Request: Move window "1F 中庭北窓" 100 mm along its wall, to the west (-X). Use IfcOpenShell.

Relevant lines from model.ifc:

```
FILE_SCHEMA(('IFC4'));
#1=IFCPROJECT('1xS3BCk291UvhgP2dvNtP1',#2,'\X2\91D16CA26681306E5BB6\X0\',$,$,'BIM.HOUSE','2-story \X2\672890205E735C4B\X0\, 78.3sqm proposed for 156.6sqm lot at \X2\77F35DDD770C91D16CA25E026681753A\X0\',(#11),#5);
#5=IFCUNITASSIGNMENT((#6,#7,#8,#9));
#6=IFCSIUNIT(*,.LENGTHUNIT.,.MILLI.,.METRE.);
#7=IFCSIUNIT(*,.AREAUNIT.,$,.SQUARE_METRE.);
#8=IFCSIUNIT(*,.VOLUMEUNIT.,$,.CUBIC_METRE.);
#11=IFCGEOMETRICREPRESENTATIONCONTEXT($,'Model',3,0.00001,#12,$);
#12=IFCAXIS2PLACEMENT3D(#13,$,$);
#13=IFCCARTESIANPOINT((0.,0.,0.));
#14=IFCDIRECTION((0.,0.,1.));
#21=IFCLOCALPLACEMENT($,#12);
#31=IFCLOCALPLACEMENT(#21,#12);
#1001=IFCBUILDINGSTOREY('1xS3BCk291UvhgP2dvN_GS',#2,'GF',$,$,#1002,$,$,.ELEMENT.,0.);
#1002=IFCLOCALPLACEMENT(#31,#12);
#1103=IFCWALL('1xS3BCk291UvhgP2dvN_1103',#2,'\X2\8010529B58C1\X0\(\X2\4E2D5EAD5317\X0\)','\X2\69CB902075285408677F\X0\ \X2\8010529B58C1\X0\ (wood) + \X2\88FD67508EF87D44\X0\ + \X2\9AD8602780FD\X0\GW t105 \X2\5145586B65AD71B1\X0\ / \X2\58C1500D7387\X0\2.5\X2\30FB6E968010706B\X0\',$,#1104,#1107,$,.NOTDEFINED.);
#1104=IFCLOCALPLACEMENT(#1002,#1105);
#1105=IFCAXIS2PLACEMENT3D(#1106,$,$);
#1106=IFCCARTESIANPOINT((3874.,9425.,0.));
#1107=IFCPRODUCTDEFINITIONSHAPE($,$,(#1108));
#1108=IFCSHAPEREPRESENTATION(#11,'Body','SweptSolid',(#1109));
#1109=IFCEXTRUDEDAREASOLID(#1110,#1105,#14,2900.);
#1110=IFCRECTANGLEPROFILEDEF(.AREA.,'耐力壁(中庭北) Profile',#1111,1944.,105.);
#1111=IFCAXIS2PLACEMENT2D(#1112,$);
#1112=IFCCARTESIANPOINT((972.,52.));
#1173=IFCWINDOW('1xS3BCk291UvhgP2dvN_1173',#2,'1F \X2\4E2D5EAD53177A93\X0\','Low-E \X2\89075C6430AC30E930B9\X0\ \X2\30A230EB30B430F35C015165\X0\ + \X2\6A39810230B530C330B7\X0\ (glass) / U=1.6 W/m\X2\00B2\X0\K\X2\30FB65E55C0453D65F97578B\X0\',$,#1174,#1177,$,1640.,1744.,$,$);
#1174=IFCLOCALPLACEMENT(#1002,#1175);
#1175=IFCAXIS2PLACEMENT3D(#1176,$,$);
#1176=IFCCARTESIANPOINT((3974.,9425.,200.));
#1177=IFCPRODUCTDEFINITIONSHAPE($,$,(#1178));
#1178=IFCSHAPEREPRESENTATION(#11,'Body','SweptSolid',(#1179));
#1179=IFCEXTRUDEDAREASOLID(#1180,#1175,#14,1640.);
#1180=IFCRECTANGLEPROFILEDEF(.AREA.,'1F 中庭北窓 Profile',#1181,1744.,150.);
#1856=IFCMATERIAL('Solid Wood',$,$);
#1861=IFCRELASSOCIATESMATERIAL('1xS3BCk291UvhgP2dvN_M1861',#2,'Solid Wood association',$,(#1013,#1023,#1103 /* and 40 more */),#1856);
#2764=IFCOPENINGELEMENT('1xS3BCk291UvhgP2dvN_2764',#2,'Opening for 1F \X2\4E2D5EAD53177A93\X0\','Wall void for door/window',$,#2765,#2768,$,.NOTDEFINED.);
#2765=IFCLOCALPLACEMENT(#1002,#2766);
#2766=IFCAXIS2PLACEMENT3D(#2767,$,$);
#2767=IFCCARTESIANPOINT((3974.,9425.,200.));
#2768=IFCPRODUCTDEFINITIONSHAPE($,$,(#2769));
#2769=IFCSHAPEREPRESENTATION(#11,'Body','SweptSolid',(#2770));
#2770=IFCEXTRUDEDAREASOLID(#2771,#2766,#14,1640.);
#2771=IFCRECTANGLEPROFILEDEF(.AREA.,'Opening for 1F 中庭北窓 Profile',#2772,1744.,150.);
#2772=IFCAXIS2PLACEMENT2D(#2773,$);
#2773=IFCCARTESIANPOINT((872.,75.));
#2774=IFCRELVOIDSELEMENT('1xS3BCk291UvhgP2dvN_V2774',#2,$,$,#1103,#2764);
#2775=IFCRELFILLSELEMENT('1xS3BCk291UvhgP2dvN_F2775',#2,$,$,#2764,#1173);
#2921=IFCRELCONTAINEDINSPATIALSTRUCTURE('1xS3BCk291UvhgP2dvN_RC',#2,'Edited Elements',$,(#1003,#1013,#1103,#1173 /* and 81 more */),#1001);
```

```python
import ifcopenshell
import ifcopenshell.api.geometry
import ifcopenshell.util.placement
import ifcopenshell.util.unit

model = ifcopenshell.open("model.ifc")
unit_scale = ifcopenshell.util.unit.calculate_unit_scale(model)

window = model.by_id(1173)
opening = window.FillsVoids[0].RelatingOpeningElement
wall = opening.VoidsElements[0].RelatingBuildingElement

wall_matrix = ifcopenshell.util.placement.get_local_placement(wall.ObjectPlacement)
shift = wall_matrix[:3, 0] * -0.1 / unit_scale
before = ifcopenshell.util.placement.get_local_placement(window.ObjectPlacement)[:3, 3].copy()

# The window is not placed relative to its opening, so move both.
for product in (opening, window):
    matrix = ifcopenshell.util.placement.get_local_placement(product.ObjectPlacement)
    matrix[:3, 3] += shift
    ifcopenshell.api.geometry.edit_object_placement(model, product=product, matrix=matrix, is_si=False)

after = ifcopenshell.util.placement.get_local_placement(window.ObjectPlacement)[:3, 3]
print("window moved by", (after - before).round(3) + 0.0)

model.write("model_rev.ifc")
```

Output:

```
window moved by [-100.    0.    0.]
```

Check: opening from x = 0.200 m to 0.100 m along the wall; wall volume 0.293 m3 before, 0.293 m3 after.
